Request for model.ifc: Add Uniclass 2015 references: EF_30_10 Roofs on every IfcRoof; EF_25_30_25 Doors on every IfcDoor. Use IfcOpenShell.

First a look at what the model holds.

```python
import ifcopenshell

model = ifcopenshell.open("model.ifc")
print(model.schema)
print("classifications:", [c.Name for c in model.by_type("IfcClassification")])
for ifc_class in ("IfcDoor", "IfcRoof", "IfcStair", "IfcWall", "IfcWindow"):
    print(ifc_class, len(model.by_type(ifc_class)))
```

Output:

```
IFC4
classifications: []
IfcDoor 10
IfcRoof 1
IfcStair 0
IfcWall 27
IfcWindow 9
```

```python
import ifcopenshell
import ifcopenshell.api.classification

model = ifcopenshell.open("model.ifc")

system = ifcopenshell.api.classification.add_classification(model, classification="Uniclass 2015")

codes = {
    "IfcRoof": ("EF_30_10", "Roofs"),
    "IfcDoor": ("EF_25_30_25", "Doors"),
}
for ifc_class, (code, name) in codes.items():
    products = model.by_type(ifc_class)
    ifcopenshell.api.classification.add_reference(
        model, products=products, classification=system, identification=code, name=name
    )
    print(code, len(products))

model.write("model-out.ifc")
```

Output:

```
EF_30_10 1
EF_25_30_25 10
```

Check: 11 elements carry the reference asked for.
